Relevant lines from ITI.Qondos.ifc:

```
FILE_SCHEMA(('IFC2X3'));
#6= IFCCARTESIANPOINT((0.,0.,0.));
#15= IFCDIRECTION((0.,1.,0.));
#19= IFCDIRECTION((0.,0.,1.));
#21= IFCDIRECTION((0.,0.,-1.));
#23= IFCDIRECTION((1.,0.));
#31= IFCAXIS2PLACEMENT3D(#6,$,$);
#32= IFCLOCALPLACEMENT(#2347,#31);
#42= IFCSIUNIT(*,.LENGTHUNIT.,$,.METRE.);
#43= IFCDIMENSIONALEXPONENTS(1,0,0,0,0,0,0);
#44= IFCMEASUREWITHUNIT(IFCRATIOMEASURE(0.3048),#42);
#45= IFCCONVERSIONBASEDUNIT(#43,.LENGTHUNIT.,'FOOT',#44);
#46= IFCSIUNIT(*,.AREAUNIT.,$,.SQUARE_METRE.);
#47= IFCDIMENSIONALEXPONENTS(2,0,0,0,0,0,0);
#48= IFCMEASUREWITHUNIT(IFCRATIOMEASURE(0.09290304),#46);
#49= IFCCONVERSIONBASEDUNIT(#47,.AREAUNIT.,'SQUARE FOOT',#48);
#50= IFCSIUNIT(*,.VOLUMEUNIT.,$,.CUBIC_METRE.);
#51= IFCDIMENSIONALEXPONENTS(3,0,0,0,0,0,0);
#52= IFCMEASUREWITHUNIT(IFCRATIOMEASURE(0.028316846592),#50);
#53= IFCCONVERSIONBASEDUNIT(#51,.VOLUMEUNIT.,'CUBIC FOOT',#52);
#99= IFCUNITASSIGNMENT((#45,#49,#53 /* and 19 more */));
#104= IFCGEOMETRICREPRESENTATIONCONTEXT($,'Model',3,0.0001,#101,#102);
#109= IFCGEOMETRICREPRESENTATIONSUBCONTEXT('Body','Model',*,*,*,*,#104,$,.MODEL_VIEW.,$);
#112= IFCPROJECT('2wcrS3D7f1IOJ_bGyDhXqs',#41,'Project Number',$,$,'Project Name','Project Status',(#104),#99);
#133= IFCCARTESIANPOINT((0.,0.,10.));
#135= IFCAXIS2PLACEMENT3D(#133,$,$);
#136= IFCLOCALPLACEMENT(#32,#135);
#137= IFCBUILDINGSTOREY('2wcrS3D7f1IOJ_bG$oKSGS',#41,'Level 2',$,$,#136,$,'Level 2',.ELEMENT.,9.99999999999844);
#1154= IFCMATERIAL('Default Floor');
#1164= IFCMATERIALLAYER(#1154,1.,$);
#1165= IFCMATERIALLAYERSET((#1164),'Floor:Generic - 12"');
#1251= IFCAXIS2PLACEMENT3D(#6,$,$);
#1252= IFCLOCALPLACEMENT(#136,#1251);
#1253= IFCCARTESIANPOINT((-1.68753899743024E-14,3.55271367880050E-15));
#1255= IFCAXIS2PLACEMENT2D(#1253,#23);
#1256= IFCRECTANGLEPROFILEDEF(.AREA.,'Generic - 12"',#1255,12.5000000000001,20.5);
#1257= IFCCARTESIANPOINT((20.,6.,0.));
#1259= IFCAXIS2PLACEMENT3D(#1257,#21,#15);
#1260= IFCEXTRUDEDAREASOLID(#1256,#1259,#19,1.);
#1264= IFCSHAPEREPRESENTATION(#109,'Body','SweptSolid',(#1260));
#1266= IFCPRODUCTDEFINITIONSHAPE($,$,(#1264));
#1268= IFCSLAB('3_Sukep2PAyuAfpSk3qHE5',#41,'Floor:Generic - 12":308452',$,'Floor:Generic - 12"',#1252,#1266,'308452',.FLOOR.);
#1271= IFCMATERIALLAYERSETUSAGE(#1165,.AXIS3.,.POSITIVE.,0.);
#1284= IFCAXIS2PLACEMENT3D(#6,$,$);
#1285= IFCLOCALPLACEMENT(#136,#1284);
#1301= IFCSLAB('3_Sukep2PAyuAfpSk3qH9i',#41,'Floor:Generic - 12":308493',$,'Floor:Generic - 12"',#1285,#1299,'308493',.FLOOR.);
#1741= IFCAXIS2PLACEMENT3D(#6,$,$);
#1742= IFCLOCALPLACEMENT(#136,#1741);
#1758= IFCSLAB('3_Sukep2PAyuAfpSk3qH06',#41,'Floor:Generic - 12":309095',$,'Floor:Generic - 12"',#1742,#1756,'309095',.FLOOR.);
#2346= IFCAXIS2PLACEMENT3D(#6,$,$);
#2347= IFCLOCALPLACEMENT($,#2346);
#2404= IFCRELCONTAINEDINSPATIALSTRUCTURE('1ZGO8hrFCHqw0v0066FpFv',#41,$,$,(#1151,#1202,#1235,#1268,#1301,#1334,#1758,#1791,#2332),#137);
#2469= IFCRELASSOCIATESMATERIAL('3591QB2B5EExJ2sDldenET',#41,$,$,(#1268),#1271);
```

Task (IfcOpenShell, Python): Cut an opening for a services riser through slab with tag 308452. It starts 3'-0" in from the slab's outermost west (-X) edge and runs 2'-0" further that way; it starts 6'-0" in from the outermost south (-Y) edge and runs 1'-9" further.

```python
import numpy as np
import ifcopenshell
import ifcopenshell.api.feature
import ifcopenshell.api.geometry
import ifcopenshell.api.root
import ifcopenshell.geom
import ifcopenshell.util.placement
import ifcopenshell.util.representation
import ifcopenshell.util.shape
import ifcopenshell.util.unit

model = ifcopenshell.open("ITI.Qondos.ifc")
unit_scale = ifcopenshell.util.unit.calculate_unit_scale(model)
settings = ifcopenshell.geom.settings()


def volume(element):
    """Net volume in cubic metres, openings subtracted."""
    shape = ifcopenshell.geom.create_shape(settings, element)
    return ifcopenshell.util.shape.get_volume(shape.geometry)


slab = model.by_guid("3_Sukep2PAyuAfpSk3qHE5")
before = volume(slab)

# Extent in the slab's own axes, in metres. The edges named are its -X and -Y sides.
slab_shape = ifcopenshell.geom.create_shape(settings, slab)
vertices = ifcopenshell.util.shape.get_vertices(slab_shape.geometry)
x_min, y_min, bottom = vertices.min(axis=0)
top = vertices[:, 2].max()

opening = ifcopenshell.api.root.create_entity(model, ifc_class="IfcOpeningElement", name="Services riser opening")
context = ifcopenshell.util.representation.get_context(model, "Model", "Body", "MODEL_VIEW")
width, depth = 0.6096, 0.5334
outline = [(0.0, 0.0), (width, 0.0), (width, depth), (0.0, depth), (0.0, 0.0)]
# Overshoot both faces by 50 mm so the cut is clean.
shape = ifcopenshell.api.geometry.add_slab_representation(
    model, context=context, depth=top - bottom + 0.1, polyline=outline
)
ifcopenshell.api.geometry.assign_representation(model, product=opening, representation=shape)

matrix = ifcopenshell.util.placement.get_local_placement(slab.ObjectPlacement)
matrix[:, 3] = matrix @ np.append(np.array([x_min + 0.9144, y_min + 1.8288, bottom - 0.05]) / unit_scale, 1.0)
ifcopenshell.api.geometry.edit_object_placement(model, product=opening, matrix=matrix, is_si=False)
ifcopenshell.api.feature.add_feature(model, feature=opening, element=slab)

after = volume(slab)

print(f"slab volume {before:.3f} -> {after:.3f} m3")

model.write("ITI.Qondos_v2.ifc")
```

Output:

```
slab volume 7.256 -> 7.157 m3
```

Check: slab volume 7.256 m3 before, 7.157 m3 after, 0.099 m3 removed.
